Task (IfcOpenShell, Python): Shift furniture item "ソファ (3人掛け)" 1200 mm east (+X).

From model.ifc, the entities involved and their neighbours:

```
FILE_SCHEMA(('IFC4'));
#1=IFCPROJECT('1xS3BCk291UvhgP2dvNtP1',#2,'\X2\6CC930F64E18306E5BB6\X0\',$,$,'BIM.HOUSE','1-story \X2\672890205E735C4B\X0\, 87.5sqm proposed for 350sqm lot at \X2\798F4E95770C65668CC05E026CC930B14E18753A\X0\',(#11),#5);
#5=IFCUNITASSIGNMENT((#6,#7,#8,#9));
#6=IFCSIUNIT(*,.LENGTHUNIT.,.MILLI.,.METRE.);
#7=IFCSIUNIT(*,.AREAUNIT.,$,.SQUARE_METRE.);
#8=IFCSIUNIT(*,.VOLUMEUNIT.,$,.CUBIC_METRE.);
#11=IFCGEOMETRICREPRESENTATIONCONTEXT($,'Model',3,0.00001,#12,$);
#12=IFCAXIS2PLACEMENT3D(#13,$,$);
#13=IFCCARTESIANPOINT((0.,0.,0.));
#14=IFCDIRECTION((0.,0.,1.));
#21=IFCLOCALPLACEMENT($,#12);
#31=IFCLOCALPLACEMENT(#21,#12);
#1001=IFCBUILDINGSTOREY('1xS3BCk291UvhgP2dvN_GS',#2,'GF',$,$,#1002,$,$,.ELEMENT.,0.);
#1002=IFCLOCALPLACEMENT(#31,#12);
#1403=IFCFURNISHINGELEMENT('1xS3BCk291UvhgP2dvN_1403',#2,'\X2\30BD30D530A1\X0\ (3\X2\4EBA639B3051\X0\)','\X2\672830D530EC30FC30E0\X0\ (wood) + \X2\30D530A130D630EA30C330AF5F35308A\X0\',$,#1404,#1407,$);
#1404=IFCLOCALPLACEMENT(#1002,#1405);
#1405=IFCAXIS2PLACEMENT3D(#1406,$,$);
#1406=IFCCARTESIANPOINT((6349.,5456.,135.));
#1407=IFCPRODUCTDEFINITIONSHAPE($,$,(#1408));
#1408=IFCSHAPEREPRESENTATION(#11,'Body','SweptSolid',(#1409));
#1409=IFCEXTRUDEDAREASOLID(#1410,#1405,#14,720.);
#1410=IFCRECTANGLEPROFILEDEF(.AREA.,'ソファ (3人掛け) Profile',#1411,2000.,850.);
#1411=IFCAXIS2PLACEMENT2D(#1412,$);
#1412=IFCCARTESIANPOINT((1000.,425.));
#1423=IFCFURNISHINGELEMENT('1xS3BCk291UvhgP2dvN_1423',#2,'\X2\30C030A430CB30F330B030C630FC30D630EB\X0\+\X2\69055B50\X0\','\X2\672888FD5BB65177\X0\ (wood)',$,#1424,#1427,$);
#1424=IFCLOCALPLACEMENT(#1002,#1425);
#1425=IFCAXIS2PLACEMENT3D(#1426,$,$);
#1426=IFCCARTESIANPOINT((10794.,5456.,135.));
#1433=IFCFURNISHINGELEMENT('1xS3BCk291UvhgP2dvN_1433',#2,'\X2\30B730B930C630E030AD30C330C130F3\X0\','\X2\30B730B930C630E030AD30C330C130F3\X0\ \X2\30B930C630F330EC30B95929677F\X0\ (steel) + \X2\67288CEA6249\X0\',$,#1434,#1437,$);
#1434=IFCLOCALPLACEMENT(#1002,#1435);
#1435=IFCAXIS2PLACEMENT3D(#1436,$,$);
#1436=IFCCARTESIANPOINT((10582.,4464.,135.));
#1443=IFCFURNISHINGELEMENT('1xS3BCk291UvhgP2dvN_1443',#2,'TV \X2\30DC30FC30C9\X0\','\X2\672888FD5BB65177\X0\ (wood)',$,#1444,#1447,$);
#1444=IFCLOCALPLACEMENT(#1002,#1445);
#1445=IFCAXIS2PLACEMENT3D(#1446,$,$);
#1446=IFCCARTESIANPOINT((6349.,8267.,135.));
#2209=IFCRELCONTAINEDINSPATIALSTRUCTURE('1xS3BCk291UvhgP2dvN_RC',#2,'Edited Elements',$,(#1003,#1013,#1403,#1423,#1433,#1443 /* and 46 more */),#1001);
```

```python
import ifcopenshell
import ifcopenshell.api.geometry
import ifcopenshell.util.placement

model = ifcopenshell.open("model.ifc")

item = model.by_guid("1xS3BCk291UvhgP2dvN_1403")
matrix = ifcopenshell.util.placement.get_local_placement(item.ObjectPlacement)
matrix[0, 3] += 1200.0
ifcopenshell.api.geometry.edit_object_placement(model, product=item, matrix=matrix, is_si=False)

print(ifcopenshell.util.placement.get_local_placement(item.ObjectPlacement).round(3) + 0.0)

model.write("model_edited.ifc")
```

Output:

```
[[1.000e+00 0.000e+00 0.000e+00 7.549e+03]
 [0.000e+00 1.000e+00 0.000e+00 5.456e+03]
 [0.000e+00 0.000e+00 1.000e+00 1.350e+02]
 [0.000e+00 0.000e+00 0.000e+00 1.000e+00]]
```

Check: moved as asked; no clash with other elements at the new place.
